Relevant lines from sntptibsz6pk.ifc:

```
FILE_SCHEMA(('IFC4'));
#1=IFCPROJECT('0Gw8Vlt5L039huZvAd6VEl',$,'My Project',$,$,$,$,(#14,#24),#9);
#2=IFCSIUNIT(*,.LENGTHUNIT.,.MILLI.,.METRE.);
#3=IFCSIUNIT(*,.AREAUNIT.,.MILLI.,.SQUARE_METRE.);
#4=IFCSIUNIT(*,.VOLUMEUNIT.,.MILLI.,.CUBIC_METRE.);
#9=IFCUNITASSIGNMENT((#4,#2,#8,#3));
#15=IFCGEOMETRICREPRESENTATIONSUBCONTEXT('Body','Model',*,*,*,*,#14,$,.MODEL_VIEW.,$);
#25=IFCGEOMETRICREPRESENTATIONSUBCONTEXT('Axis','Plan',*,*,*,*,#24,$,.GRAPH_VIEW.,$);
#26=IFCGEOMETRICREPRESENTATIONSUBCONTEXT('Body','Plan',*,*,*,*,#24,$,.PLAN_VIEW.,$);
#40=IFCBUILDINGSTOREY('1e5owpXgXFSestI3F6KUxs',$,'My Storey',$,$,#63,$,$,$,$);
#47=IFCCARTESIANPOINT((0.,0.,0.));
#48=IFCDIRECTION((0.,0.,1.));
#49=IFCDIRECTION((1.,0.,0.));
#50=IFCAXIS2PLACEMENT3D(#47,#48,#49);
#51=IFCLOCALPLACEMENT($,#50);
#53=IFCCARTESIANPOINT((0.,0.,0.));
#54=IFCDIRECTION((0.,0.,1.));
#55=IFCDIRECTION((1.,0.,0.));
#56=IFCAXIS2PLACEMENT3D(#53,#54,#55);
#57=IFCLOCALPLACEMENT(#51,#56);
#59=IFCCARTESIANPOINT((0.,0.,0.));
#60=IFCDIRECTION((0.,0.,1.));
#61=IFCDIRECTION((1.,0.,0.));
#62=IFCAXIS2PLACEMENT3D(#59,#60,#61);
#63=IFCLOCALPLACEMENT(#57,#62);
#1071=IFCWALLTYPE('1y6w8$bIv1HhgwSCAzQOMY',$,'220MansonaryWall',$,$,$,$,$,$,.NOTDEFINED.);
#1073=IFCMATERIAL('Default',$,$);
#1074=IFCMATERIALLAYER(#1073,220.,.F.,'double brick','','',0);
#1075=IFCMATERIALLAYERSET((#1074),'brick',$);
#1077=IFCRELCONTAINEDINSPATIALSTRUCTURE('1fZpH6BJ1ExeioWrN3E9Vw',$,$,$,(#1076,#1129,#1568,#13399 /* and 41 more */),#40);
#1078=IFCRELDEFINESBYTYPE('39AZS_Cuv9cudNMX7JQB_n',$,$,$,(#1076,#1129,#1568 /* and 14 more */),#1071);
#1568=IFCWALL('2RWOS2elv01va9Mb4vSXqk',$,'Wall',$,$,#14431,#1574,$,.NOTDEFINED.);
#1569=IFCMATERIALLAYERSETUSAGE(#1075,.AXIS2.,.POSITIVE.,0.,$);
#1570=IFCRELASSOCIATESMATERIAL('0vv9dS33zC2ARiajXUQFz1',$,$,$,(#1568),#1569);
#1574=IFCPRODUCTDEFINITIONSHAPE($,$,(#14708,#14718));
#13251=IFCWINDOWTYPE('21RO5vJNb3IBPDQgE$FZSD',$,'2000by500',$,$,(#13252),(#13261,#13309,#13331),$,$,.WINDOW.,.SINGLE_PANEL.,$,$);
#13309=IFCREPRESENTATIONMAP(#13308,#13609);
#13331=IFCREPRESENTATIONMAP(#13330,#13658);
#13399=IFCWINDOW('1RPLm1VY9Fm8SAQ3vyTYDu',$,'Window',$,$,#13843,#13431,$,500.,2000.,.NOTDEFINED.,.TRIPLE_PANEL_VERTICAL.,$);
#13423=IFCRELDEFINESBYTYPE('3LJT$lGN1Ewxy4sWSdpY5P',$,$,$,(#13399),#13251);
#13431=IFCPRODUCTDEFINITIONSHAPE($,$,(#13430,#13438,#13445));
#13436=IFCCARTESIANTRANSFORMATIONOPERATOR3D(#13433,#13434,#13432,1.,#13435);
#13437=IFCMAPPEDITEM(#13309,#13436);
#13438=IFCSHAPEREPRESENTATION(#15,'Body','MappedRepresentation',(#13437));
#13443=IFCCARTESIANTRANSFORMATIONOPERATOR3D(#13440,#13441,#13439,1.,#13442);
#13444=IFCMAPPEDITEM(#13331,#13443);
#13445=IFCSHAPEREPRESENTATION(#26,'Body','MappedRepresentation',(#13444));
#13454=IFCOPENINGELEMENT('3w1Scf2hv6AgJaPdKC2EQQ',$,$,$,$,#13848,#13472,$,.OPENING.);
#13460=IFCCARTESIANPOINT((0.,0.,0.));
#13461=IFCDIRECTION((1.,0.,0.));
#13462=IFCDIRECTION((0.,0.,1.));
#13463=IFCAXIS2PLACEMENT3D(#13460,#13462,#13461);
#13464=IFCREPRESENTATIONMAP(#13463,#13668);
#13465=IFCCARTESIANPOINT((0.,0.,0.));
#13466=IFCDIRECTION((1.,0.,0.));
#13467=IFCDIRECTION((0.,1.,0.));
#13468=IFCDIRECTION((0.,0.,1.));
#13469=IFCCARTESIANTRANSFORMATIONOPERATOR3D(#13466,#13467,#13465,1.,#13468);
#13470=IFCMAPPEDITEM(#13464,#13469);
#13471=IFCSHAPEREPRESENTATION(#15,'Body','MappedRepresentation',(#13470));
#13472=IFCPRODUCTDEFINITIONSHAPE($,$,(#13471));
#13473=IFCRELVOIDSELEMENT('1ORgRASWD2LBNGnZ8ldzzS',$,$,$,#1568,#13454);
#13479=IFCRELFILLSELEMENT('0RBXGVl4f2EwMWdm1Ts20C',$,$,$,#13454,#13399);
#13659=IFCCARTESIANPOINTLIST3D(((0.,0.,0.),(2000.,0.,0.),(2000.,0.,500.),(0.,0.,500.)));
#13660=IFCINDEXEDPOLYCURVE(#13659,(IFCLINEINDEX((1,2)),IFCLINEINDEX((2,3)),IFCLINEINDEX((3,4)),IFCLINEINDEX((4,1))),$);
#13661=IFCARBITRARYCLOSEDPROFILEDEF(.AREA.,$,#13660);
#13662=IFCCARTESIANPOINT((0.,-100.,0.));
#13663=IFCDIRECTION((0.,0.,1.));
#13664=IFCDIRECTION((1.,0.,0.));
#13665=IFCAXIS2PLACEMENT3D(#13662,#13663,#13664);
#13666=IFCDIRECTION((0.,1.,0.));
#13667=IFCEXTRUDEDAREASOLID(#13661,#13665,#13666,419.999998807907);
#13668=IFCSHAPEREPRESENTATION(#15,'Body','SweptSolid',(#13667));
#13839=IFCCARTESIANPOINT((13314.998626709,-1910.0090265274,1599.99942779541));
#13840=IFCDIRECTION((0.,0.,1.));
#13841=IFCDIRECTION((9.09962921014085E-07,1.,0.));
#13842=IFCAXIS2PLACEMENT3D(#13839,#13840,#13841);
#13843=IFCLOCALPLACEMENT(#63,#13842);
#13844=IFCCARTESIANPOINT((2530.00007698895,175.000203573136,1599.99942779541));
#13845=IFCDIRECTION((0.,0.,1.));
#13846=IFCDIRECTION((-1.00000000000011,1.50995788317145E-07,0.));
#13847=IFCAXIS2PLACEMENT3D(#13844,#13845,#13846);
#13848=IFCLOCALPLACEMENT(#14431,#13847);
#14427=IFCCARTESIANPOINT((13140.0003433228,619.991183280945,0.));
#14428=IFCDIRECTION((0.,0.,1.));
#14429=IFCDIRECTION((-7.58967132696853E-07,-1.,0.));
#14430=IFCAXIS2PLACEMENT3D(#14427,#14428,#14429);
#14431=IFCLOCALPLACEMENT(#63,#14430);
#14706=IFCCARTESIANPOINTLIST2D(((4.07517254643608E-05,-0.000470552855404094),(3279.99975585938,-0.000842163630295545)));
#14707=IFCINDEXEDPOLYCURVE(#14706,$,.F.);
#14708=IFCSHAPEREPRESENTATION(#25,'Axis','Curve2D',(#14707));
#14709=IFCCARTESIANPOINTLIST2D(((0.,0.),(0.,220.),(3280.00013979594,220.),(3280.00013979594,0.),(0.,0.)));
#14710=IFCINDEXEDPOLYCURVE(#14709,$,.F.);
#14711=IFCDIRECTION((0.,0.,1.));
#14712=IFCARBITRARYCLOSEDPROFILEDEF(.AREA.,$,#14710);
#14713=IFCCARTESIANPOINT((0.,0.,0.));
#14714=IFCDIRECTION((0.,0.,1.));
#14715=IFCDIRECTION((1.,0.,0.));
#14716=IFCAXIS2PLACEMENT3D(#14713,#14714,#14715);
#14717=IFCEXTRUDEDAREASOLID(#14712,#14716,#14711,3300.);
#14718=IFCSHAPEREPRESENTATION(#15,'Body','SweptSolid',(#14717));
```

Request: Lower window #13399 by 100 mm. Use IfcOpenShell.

```python
import numpy as np
import ifcopenshell
import ifcopenshell.api.geometry
import ifcopenshell.util.placement
import ifcopenshell.util.unit

model = ifcopenshell.open("sntptibsz6pk.ifc")
unit_scale = ifcopenshell.util.unit.calculate_unit_scale(model)

window = model.by_guid("1RPLm1VY9Fm8SAQ3vyTYDu")
opening = window.FillsVoids[0].RelatingOpeningElement
dz = -0.1 / unit_scale

shift = np.array([0.0, 0.0, dz])
# The window is not placed relative to its opening, so move both.
for product in (opening, window):
    matrix = ifcopenshell.util.placement.get_local_placement(product.ObjectPlacement)
    matrix[:3, 3] += shift
    ifcopenshell.api.geometry.edit_object_placement(model, product=product, matrix=matrix, is_si=False)

print(f"moved by {dz * unit_scale:+.3f} m")

model.write("sntptibsz6pk_v2.ifc")
```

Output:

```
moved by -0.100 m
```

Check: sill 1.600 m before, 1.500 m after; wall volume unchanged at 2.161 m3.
